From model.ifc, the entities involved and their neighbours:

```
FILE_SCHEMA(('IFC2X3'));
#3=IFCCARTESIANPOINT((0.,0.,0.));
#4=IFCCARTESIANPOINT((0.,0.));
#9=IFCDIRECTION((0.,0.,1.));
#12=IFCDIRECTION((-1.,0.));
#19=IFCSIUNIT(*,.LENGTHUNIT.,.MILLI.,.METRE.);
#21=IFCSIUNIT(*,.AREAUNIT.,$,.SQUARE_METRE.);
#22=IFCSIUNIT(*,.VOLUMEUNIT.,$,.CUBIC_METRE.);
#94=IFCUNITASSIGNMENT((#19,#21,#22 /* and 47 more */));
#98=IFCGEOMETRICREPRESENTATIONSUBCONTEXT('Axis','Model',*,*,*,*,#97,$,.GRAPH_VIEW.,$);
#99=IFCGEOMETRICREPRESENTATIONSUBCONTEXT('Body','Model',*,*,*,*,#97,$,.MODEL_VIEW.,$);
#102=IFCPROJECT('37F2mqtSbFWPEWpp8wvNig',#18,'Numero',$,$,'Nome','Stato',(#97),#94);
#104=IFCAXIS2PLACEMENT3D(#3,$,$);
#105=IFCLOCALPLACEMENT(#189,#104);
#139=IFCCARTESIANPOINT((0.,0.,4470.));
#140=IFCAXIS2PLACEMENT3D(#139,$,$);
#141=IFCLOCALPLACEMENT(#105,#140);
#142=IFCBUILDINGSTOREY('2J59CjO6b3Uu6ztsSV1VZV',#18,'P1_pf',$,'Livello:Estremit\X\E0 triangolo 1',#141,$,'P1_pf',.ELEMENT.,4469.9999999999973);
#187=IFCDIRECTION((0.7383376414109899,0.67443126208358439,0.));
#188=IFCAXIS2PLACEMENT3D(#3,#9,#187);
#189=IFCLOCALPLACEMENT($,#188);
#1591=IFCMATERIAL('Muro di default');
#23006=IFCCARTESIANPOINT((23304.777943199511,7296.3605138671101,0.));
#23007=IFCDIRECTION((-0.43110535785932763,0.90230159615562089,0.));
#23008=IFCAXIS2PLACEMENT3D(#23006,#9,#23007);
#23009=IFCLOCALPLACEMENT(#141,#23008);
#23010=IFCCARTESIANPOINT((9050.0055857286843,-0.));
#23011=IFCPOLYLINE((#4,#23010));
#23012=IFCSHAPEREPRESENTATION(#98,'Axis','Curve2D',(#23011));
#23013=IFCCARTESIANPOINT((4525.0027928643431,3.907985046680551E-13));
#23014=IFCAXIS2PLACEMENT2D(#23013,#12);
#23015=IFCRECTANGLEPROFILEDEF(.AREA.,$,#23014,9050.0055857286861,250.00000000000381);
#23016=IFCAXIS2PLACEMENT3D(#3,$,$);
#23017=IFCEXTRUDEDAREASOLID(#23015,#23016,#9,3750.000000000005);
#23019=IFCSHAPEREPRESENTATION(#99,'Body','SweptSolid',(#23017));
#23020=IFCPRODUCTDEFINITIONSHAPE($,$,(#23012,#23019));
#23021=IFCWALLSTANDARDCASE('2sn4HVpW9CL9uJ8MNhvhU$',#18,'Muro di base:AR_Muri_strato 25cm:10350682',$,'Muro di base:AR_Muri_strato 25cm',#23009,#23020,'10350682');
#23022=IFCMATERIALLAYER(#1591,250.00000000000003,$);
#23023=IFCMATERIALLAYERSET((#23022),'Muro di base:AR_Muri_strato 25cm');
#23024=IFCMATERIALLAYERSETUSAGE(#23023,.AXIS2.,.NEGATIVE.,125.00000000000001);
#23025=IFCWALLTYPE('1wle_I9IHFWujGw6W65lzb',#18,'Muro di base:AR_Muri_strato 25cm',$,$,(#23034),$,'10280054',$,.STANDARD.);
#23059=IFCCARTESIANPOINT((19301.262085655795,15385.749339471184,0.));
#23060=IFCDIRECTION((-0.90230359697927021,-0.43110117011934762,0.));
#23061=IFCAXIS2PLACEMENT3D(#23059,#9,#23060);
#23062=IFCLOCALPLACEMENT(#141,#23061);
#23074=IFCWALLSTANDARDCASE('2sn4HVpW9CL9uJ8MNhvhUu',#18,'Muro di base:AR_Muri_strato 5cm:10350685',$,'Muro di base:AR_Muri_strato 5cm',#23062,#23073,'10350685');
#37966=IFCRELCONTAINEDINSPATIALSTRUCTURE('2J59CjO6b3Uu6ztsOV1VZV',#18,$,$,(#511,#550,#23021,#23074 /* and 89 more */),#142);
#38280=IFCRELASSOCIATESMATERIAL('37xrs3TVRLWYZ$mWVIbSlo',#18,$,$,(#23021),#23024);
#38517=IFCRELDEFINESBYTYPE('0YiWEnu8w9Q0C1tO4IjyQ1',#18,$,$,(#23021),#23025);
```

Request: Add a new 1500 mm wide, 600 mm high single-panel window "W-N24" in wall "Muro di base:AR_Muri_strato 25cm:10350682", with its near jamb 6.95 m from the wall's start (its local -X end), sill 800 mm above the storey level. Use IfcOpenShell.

```python
import numpy as np
import ifcopenshell
import ifcopenshell.api.feature
import ifcopenshell.api.geometry
import ifcopenshell.api.root
import ifcopenshell.api.spatial
import ifcopenshell.api.type
import ifcopenshell.geom
import ifcopenshell.util.element
import ifcopenshell.util.placement
import ifcopenshell.util.representation
import ifcopenshell.util.shape
import ifcopenshell.util.unit

model = ifcopenshell.open("model.ifc")
unit_scale = ifcopenshell.util.unit.calculate_unit_scale(model)
settings = ifcopenshell.geom.settings()


def volume(element):
    """Net volume in cubic metres, openings subtracted."""
    shape = ifcopenshell.geom.create_shape(settings, element)
    return ifcopenshell.util.shape.get_volume(shape.geometry)


wall = model.by_id(23021)
storey = ifcopenshell.util.element.get_container(wall, ifc_class="IfcBuildingStorey")
context = ifcopenshell.util.representation.get_context(model, "Model", "Body", "MODEL_VIEW")
before = volume(wall)

width, height, from_end, sill = 1.5, 0.6, 6.95, 0.8  # metres

# The wall runs along its own X axis, and the end named is its -X end.
wall_shape = ifcopenshell.geom.create_shape(settings, wall)
x, y, z = ifcopenshell.util.shape.get_vertices(wall_shape.geometry).T
start = x.min() + from_end
face, thickness = float(y.min()), float(y.max() - y.min())
wall_matrix = ifcopenshell.util.placement.get_local_placement(wall.ObjectPlacement)
level = ifcopenshell.util.placement.get_local_placement(storey.ObjectPlacement)[2, 3]


def in_wall(x, y):
    """Placement at x, y metres in the wall's axes, at sill height."""
    matrix = wall_matrix.copy()
    matrix[:, 3] = wall_matrix @ np.array([x / unit_scale, y / unit_scale, 0.0, 1.0])
    matrix[2, 3] = level + sill / unit_scale
    return matrix


# Opening: a box that overshoots both wall faces by 50 mm.
opening = ifcopenshell.api.root.create_entity(model, ifc_class="IfcOpeningElement")
box = ifcopenshell.api.geometry.add_wall_representation(
    model, context=context, length=width, height=height, thickness=thickness + 0.1
)
ifcopenshell.api.geometry.assign_representation(model, product=opening, representation=box)
ifcopenshell.api.geometry.edit_object_placement(model, product=opening, matrix=in_wall(start, face - 0.05), is_si=False)
ifcopenshell.api.feature.add_feature(model, feature=opening, element=wall)

window = ifcopenshell.api.root.create_entity(model, ifc_class="IfcWindow", name="W-N24")
window.OverallWidth, window.OverallHeight = width / unit_scale, height / unit_scale
body = ifcopenshell.api.geometry.add_window_representation(
    model,
    context=context,
    overall_width=window.OverallWidth,
    overall_height=window.OverallHeight,
    partition_type="SINGLE_PANEL",
)
ifcopenshell.api.geometry.assign_representation(model, product=window, representation=body)
ifcopenshell.api.spatial.assign_container(model, products=[window], relating_structure=storey)
fills = ifcopenshell.api.feature.add_filling(model, opening=opening, element=window)
fills.OwnerHistory = window.OwnerHistory  # required in IFC2X3

# IFC2X3 keeps the operation on the window style.
style = ifcopenshell.api.root.create_entity(model, ifc_class="IfcWindowStyle", name="W-N24")
style.OperationType, style.ConstructionType = "SINGLE_PANEL", "NOTDEFINED"
style.ParameterTakesPrecedence = style.Sizeable = False
ifcopenshell.api.type.assign_type(model, related_objects=[window], relating_type=style)

# Centre the window in the wall's thickness.
ifcopenshell.api.geometry.edit_object_placement(model, product=window, matrix=in_wall(start, face), is_si=False)
window_shape = ifcopenshell.geom.create_shape(settings, window)
depth = ifcopenshell.util.shape.get_vertices(window_shape.geometry)[:, 1]
offset = face + thickness / 2 - (depth.min() + depth.max()) / 2
ifcopenshell.api.geometry.edit_object_placement(model, product=window, matrix=in_wall(start, offset), is_si=False)

after = volume(wall)

print(f"wall volume {before:.3f} -> {after:.3f} m3")

model.write("model_v2.ifc")
```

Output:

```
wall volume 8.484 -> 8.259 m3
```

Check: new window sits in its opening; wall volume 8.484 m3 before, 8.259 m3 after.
